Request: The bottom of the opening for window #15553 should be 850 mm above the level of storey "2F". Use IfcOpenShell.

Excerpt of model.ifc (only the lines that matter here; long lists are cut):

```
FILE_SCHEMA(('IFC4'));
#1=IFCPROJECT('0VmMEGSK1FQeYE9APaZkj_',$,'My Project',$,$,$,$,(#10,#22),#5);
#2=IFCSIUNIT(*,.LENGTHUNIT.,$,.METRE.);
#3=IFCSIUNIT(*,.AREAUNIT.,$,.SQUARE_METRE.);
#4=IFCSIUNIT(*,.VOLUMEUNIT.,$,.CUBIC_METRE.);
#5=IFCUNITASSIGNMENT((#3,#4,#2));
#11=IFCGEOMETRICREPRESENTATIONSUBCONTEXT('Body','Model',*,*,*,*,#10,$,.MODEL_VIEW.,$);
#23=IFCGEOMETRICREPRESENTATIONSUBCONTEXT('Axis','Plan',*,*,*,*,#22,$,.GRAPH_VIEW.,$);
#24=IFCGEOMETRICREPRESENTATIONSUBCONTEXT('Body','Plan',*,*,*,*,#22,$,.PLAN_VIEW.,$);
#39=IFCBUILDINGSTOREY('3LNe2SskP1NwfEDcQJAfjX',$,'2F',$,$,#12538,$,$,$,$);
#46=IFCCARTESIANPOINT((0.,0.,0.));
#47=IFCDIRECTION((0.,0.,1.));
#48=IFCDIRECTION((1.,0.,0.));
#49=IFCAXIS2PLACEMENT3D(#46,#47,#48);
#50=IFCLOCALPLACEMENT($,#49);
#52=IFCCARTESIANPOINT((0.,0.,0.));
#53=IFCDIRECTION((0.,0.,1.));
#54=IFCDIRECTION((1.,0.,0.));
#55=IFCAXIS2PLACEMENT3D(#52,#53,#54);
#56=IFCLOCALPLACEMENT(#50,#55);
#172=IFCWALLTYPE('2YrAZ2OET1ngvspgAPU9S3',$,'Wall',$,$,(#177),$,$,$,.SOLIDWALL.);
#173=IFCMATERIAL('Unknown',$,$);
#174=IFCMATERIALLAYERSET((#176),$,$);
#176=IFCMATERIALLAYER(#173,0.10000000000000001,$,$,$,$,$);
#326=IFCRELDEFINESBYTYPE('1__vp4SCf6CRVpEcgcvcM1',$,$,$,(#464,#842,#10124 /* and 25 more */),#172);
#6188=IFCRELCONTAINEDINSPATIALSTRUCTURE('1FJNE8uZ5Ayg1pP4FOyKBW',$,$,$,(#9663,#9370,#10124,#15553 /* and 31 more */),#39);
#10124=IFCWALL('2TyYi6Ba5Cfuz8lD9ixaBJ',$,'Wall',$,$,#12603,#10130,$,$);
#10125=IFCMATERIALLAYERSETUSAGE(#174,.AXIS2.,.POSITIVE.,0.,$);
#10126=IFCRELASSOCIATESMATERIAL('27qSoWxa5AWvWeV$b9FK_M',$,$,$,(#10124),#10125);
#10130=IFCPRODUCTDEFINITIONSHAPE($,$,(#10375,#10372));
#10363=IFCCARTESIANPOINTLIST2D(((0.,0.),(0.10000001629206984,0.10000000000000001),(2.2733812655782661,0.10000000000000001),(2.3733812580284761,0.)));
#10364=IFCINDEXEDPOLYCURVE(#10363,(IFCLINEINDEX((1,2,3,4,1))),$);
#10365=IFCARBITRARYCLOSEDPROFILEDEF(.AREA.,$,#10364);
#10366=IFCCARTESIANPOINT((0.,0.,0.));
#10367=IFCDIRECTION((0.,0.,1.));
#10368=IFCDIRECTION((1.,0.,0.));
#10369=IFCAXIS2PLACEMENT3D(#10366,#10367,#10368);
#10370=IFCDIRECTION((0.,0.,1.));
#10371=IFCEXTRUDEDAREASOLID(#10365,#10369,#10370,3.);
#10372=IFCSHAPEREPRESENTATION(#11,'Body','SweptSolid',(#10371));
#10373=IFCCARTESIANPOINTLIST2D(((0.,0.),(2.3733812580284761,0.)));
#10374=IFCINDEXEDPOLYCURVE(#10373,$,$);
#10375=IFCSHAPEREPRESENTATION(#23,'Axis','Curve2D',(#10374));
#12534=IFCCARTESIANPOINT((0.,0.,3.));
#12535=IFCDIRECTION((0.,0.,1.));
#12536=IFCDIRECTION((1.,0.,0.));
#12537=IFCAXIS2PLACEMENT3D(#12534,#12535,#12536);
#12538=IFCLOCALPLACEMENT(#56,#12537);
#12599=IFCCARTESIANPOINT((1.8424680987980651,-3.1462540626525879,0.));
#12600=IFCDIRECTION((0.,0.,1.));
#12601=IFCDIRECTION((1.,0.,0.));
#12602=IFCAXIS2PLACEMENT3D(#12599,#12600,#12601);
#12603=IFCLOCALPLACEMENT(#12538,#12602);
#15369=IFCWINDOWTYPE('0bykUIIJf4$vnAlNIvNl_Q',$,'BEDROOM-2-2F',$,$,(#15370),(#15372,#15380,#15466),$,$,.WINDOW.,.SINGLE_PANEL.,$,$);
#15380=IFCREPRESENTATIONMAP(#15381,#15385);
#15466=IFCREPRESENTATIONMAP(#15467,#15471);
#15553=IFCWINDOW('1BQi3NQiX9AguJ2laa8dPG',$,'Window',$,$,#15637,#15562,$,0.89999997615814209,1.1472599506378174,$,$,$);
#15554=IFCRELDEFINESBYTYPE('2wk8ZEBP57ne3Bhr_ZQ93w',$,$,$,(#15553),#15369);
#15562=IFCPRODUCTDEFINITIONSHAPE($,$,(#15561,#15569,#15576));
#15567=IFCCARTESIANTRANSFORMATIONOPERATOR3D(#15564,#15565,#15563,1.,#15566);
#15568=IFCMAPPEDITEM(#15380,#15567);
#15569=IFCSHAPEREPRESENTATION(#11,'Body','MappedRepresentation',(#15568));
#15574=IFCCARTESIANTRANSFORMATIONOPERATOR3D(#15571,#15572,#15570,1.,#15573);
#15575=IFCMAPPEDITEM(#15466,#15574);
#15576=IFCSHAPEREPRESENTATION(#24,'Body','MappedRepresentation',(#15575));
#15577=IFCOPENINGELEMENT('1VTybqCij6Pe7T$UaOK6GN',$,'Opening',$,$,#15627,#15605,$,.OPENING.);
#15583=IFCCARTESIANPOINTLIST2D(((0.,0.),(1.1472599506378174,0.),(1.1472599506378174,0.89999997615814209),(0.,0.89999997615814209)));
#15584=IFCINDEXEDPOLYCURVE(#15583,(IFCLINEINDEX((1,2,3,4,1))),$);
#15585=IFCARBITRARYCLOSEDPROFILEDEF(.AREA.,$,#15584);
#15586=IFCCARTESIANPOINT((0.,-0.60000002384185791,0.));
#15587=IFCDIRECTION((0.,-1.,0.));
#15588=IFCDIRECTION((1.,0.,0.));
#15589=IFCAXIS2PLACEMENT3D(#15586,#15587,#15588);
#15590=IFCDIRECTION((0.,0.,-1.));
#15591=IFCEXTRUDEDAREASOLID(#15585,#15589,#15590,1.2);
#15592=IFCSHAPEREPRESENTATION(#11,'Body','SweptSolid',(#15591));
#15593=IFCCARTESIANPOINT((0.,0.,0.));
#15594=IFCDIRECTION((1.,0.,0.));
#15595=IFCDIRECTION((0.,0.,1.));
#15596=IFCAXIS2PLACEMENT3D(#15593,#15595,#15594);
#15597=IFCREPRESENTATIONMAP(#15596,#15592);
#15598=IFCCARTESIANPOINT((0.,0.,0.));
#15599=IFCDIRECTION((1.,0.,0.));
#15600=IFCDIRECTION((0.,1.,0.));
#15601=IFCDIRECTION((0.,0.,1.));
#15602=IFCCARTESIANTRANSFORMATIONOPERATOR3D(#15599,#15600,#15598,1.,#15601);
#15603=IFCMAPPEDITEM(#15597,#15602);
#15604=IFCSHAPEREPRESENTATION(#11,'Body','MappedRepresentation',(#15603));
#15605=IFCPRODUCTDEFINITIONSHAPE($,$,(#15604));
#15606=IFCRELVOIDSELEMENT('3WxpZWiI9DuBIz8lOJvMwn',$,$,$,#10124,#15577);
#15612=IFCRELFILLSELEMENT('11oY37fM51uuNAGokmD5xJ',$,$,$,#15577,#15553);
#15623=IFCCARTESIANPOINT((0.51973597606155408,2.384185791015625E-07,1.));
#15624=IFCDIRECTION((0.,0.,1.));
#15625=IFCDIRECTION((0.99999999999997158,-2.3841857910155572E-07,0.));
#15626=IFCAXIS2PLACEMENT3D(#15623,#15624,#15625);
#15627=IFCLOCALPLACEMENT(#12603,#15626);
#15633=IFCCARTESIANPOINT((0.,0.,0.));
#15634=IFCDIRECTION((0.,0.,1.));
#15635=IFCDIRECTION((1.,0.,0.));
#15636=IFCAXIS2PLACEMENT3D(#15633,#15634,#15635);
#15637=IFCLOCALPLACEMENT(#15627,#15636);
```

```python
import numpy as np
import ifcopenshell
import ifcopenshell.api.geometry
import ifcopenshell.geom
import ifcopenshell.util.element
import ifcopenshell.util.placement
import ifcopenshell.util.shape
import ifcopenshell.util.unit

model = ifcopenshell.open("model.ifc")
unit_scale = ifcopenshell.util.unit.calculate_unit_scale(model)

window = model.by_guid("1BQi3NQiX9AguJ2laa8dPG")
opening = window.FillsVoids[0].RelatingOpeningElement
storey = ifcopenshell.util.element.get_container(window, ifc_class="IfcBuildingStorey")
level = ifcopenshell.util.placement.get_local_placement(storey.ObjectPlacement)[2, 3]

# The opening's origin need not be at the sill, so measure its lowest point.
shape = ifcopenshell.geom.create_shape(ifcopenshell.geom.settings(), opening)
bottom = ifcopenshell.util.shape.get_shape_bottom_elevation(shape, shape.geometry) / unit_scale
dz = level + 0.85 / unit_scale - bottom

shift = np.array([0.0, 0.0, dz])
# The window is placed relative to its opening, so it follows when the opening moves.
matrix = ifcopenshell.util.placement.get_local_placement(opening.ObjectPlacement)
matrix[:3, 3] += shift
ifcopenshell.api.geometry.edit_object_placement(
    model, product=opening, matrix=matrix, is_si=False, should_transform_children=True
)

print(f"moved by {dz * unit_scale:+.3f} m")

model.write("model_edited.ifc")
```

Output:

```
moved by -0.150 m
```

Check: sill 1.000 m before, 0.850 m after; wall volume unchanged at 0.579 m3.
